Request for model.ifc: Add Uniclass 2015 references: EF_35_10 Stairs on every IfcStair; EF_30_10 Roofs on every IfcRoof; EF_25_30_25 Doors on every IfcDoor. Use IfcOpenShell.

First a look at what the model holds.

```python
import ifcopenshell

model = ifcopenshell.open("model.ifc")
print(model.schema)
print("classifications:", [c.Name for c in model.by_type("IfcClassification")])
for ifc_class in ("IfcDoor", "IfcRoof", "IfcStair", "IfcWall", "IfcWindow"):
    print(ifc_class, len(model.by_type(ifc_class)))
```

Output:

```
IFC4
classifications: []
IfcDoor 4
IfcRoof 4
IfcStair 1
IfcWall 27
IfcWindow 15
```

```python
import ifcopenshell
import ifcopenshell.api.classification

model = ifcopenshell.open("model.ifc")

system = ifcopenshell.api.classification.add_classification(model, classification="Uniclass 2015")

codes = {
    "IfcStair": ("EF_35_10", "Stairs"),
    "IfcRoof": ("EF_30_10", "Roofs"),
    "IfcDoor": ("EF_25_30_25", "Doors"),
}
for ifc_class, (code, name) in codes.items():
    products = model.by_type(ifc_class)
    ifcopenshell.api.classification.add_reference(
        model, products=products, classification=system, identification=code, name=name
    )
    print(code, len(products))

model.write("model_v2.ifc")
```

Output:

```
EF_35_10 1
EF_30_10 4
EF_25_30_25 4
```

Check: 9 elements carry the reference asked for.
